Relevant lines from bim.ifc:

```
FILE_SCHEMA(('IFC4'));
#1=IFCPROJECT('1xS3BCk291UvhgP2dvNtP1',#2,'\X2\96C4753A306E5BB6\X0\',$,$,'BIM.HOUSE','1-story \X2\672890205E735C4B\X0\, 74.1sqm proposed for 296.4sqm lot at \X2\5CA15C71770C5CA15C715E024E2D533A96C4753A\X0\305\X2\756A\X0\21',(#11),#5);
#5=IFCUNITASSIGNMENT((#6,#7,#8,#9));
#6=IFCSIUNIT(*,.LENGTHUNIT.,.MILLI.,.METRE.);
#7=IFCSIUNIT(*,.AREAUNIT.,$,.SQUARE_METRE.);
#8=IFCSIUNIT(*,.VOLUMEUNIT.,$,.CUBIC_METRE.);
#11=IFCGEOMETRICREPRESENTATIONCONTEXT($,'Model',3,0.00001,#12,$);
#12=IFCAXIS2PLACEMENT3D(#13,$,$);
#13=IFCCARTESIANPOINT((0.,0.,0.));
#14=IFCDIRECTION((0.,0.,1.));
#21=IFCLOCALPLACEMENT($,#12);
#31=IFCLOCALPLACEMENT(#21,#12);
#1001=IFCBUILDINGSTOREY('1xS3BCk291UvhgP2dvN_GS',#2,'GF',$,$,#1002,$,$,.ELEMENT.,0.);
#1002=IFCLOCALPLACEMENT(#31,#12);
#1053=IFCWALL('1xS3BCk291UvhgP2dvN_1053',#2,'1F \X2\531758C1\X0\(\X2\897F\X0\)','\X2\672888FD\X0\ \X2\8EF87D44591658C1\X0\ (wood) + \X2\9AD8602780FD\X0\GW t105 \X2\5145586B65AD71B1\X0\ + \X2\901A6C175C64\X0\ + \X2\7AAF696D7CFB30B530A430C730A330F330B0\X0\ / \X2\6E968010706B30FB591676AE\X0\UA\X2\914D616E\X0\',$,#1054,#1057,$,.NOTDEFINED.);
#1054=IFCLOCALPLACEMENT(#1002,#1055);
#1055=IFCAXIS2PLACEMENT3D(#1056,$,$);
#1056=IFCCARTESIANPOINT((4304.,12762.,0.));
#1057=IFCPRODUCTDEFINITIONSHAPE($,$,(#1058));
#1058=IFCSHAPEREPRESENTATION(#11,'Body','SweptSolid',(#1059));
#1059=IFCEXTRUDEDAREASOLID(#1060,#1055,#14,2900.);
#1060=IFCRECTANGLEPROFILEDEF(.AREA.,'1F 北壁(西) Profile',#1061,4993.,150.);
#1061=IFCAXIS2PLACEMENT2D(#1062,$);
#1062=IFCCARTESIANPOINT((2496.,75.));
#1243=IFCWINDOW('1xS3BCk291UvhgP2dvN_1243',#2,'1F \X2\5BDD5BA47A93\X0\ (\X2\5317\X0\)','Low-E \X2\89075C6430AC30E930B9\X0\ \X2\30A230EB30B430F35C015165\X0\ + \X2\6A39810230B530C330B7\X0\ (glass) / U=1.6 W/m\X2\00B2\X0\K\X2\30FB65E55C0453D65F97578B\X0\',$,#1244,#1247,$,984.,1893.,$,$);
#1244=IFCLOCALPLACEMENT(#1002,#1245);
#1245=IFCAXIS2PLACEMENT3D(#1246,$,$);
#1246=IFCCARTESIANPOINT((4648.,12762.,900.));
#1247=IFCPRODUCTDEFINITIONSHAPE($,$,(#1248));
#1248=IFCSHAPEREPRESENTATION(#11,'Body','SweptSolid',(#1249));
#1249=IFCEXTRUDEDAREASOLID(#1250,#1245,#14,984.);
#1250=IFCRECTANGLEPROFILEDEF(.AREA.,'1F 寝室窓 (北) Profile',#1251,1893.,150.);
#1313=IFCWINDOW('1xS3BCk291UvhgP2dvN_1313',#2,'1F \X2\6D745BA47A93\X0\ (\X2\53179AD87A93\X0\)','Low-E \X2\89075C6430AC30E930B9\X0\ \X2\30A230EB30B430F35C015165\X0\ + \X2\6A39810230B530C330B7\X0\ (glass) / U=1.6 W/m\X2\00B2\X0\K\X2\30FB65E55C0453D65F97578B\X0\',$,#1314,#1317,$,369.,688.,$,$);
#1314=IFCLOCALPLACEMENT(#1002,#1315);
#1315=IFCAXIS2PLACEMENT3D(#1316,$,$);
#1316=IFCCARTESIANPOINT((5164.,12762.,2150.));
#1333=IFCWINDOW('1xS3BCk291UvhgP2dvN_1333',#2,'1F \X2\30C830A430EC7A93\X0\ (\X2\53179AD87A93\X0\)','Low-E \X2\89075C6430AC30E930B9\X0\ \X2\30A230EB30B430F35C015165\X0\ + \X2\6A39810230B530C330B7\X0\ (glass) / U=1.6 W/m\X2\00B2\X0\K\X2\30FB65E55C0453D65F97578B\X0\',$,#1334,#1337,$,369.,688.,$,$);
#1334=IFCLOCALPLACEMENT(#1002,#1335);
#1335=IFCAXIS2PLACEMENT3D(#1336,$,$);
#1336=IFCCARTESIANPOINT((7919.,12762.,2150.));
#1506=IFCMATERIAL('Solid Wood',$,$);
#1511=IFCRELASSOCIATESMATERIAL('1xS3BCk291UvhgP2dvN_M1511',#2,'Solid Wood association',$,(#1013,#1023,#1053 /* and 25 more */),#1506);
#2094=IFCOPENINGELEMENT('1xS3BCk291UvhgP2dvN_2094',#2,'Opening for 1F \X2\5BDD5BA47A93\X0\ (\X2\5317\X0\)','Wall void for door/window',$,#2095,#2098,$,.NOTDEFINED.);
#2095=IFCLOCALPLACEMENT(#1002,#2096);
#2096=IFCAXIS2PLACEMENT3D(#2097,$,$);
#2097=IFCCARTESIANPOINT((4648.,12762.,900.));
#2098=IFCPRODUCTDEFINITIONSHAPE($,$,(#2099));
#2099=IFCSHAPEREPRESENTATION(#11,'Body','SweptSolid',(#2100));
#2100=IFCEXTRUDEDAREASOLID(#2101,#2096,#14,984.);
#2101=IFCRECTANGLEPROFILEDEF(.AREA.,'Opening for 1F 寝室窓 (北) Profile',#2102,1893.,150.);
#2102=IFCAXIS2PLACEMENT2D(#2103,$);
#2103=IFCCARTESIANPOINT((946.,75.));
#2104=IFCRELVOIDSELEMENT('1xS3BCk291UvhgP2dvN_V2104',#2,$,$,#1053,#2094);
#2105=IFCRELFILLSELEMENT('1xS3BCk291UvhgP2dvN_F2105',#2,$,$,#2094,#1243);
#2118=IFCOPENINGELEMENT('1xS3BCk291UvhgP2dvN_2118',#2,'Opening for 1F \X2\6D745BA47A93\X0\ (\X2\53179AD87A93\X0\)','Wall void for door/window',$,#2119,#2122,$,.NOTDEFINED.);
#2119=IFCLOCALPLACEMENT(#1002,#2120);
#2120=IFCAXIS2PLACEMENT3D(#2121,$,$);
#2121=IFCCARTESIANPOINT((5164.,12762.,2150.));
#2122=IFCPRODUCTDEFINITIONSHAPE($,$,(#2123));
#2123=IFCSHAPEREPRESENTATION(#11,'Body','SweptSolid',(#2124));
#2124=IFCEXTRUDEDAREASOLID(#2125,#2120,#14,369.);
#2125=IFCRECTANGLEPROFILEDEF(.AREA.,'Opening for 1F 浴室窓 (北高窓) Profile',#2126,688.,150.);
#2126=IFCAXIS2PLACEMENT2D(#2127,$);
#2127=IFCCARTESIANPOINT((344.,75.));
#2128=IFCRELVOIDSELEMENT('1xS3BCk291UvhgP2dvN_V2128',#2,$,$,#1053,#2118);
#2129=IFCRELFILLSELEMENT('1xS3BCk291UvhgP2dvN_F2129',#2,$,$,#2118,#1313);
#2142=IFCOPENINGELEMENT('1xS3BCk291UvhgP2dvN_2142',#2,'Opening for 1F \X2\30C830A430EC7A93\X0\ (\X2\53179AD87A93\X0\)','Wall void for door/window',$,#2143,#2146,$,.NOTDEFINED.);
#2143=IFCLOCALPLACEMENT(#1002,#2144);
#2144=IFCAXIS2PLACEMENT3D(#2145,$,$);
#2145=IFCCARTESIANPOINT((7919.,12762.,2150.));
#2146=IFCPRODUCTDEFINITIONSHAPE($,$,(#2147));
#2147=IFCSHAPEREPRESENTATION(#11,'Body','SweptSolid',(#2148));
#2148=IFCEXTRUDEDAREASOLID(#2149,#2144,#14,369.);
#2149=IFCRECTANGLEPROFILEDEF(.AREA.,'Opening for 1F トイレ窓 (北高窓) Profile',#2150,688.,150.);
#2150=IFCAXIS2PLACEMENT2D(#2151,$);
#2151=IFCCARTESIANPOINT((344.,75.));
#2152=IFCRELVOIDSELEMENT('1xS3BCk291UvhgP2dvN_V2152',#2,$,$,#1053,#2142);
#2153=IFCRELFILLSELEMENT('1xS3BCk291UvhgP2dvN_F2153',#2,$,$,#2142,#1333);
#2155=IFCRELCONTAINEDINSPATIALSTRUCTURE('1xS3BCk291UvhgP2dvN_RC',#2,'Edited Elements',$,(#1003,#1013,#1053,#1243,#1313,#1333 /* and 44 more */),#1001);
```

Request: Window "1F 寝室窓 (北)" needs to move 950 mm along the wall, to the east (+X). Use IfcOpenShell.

```python
import ifcopenshell
import ifcopenshell.api.geometry
import ifcopenshell.util.placement
import ifcopenshell.util.unit

model = ifcopenshell.open("bim.ifc")
unit_scale = ifcopenshell.util.unit.calculate_unit_scale(model)

window = model.by_guid("1xS3BCk291UvhgP2dvN_1243")
opening = window.FillsVoids[0].RelatingOpeningElement
wall = opening.VoidsElements[0].RelatingBuildingElement

wall_matrix = ifcopenshell.util.placement.get_local_placement(wall.ObjectPlacement)
shift = wall_matrix[:3, 0] * 0.95 / unit_scale
before = ifcopenshell.util.placement.get_local_placement(window.ObjectPlacement)[:3, 3].copy()

# The window is not placed relative to its opening, so move both.
for product in (opening, window):
    matrix = ifcopenshell.util.placement.get_local_placement(product.ObjectPlacement)
    matrix[:3, 3] += shift
    ifcopenshell.api.geometry.edit_object_placement(model, product=product, matrix=matrix, is_si=False)

after = ifcopenshell.util.placement.get_local_placement(window.ObjectPlacement)[:3, 3]
print("window moved by", (after - before).round(3) + 0.0)

model.write("bim_rev.ifc")
```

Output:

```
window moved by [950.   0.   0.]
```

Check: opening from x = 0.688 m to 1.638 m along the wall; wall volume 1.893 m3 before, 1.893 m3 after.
